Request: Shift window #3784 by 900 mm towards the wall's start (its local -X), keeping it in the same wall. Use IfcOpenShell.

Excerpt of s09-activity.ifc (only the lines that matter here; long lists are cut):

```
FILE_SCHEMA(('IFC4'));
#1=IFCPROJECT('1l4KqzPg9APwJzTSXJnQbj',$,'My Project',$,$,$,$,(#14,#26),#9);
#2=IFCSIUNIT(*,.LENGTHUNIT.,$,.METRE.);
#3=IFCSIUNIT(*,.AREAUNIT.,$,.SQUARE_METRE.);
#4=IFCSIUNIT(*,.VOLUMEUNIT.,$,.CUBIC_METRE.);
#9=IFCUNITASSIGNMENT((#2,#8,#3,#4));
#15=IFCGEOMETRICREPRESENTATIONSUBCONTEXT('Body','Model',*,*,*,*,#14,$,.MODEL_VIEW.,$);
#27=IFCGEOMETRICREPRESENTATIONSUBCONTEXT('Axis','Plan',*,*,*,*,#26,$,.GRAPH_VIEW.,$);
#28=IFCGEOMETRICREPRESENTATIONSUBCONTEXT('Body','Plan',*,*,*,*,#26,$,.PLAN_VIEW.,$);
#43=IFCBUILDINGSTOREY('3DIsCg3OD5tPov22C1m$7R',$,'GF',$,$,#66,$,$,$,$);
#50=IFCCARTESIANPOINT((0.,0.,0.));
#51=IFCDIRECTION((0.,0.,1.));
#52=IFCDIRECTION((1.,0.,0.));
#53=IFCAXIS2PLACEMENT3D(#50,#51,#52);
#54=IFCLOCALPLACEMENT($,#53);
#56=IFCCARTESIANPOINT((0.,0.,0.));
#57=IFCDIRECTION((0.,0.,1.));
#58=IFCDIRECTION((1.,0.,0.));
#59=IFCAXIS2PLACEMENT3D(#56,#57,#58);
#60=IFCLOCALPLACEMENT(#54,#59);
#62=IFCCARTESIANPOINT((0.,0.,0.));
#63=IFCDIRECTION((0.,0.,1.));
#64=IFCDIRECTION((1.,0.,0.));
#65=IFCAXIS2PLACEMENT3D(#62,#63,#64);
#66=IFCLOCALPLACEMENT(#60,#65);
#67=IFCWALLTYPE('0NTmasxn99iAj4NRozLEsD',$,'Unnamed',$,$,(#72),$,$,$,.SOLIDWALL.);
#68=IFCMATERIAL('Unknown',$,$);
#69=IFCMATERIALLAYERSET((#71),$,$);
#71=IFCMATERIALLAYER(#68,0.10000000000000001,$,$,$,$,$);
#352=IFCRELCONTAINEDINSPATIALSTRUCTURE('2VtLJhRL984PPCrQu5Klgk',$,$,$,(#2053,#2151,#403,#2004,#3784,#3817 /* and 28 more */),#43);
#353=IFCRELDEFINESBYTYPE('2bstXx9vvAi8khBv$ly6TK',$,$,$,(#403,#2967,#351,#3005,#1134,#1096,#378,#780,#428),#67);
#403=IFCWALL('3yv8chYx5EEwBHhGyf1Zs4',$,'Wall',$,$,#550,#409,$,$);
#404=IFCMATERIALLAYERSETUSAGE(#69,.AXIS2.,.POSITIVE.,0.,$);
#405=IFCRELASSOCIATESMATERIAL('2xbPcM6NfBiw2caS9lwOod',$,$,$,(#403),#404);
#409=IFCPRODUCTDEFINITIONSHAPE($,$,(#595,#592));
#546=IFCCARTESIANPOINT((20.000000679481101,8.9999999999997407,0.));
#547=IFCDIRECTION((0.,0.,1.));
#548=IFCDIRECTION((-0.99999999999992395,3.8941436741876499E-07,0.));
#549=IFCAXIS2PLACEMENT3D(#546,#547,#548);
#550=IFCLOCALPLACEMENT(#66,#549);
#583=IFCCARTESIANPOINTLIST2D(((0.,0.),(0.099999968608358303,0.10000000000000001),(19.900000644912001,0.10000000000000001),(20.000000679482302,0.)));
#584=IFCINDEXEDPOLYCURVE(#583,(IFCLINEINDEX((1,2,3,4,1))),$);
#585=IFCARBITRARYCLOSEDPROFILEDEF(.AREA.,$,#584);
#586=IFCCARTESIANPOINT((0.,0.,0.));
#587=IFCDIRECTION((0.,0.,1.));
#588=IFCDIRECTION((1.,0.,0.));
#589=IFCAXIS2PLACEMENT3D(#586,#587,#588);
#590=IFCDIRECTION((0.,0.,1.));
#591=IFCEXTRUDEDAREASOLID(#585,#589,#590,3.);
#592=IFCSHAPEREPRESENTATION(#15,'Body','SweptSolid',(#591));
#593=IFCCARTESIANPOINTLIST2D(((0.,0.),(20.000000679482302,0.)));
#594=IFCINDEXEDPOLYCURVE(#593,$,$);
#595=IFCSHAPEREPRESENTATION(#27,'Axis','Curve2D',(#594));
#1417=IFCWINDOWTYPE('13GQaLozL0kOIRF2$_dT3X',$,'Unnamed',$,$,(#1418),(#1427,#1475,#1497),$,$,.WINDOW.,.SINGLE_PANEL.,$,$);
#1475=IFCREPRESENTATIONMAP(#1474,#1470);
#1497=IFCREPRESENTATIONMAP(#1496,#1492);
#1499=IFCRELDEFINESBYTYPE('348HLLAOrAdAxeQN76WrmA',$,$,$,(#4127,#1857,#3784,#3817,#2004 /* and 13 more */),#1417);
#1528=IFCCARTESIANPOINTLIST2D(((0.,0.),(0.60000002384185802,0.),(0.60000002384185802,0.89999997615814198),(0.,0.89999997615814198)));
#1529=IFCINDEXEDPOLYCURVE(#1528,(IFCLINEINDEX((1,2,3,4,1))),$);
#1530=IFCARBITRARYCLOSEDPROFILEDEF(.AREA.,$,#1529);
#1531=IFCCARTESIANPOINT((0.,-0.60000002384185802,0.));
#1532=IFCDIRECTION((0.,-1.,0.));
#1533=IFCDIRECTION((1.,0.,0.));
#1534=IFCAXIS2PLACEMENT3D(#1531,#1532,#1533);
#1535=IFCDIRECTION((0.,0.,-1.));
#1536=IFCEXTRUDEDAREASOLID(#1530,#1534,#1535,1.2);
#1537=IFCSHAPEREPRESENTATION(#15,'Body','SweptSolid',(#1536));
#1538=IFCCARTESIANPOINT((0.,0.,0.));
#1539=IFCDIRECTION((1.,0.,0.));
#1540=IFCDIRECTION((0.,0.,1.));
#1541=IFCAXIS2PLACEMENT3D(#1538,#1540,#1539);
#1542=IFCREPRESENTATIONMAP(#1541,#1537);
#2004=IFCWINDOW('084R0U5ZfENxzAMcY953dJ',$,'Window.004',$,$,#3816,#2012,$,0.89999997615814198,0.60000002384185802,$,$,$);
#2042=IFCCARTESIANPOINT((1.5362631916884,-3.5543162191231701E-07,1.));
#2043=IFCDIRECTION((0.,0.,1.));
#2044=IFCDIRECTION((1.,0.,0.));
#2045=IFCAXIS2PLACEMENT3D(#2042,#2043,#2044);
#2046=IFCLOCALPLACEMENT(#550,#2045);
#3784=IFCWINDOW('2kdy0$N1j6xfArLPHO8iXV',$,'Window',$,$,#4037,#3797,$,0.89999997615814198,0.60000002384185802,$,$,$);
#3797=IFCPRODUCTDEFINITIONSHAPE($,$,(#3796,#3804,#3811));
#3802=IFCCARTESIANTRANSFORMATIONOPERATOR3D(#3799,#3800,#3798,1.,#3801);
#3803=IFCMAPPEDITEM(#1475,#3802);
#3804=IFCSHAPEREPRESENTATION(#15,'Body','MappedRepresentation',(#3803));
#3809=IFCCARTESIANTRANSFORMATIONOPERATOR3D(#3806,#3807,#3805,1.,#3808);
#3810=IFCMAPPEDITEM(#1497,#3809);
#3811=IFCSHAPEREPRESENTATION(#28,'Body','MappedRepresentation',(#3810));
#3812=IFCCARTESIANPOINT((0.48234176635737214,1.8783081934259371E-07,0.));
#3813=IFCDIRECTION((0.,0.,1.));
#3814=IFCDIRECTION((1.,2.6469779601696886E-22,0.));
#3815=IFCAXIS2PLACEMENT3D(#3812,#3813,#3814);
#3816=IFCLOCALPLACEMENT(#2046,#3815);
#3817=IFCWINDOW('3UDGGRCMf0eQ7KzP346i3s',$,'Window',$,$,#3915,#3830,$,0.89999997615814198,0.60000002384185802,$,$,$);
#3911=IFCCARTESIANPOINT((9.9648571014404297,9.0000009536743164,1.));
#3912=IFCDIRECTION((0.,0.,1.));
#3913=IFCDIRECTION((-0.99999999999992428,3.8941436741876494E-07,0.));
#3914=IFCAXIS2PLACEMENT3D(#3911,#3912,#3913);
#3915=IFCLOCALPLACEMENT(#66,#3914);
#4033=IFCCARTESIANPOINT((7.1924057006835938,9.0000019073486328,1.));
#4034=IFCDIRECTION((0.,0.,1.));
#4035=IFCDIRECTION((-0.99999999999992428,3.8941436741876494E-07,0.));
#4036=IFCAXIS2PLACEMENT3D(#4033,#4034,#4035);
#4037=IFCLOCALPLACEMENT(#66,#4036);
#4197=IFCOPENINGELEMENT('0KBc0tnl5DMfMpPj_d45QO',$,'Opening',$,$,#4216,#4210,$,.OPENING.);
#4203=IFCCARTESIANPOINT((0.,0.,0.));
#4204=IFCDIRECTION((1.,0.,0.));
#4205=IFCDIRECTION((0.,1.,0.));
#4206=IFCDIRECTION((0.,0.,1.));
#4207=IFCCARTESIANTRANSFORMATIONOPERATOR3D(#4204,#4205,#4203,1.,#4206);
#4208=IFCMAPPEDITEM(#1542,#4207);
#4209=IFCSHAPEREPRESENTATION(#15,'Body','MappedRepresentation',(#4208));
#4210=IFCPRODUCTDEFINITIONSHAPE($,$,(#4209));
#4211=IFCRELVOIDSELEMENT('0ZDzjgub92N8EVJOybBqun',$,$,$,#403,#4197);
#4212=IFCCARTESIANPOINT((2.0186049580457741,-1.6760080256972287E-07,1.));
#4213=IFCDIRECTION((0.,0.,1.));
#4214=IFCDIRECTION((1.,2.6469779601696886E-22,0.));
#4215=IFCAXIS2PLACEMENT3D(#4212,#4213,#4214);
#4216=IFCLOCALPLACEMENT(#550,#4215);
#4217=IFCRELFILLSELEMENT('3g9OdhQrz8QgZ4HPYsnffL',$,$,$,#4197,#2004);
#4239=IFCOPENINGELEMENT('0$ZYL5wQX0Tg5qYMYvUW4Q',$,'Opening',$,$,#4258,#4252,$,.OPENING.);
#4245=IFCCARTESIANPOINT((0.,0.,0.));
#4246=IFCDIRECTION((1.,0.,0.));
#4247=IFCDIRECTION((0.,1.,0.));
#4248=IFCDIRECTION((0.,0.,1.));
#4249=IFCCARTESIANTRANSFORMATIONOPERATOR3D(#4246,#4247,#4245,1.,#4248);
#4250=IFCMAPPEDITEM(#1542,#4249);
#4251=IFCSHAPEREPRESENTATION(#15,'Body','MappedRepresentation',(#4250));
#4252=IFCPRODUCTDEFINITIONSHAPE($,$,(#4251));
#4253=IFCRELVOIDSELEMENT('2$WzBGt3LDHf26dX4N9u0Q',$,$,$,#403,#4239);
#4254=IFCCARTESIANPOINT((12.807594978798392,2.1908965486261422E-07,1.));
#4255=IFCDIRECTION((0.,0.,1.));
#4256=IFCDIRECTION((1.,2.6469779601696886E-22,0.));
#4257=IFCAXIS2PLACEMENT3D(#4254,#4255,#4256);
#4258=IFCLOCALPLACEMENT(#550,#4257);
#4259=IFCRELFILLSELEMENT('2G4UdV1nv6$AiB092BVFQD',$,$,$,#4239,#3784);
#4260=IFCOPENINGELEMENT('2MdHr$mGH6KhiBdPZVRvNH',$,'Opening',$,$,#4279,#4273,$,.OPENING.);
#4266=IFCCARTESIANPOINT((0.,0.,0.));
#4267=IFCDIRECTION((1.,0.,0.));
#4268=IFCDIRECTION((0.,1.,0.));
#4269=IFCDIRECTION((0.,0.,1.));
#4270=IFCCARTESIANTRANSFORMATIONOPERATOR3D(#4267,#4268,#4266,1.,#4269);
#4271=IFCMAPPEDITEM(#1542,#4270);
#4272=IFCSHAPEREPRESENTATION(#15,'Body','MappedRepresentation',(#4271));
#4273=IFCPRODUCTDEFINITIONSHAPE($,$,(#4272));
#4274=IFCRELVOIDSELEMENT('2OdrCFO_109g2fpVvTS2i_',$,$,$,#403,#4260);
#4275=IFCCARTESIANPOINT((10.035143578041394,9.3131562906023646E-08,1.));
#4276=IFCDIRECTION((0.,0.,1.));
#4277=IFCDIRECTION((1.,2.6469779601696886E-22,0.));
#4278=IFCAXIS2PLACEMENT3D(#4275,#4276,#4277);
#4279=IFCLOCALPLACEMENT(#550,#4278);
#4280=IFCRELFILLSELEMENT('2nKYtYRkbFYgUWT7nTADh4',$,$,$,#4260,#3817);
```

```python
import ifcopenshell
import ifcopenshell.api.geometry
import ifcopenshell.util.placement
import ifcopenshell.util.unit

model = ifcopenshell.open("s09-activity.ifc")
unit_scale = ifcopenshell.util.unit.calculate_unit_scale(model)

window = model.by_guid("2kdy0$N1j6xfArLPHO8iXV")
opening = window.FillsVoids[0].RelatingOpeningElement
wall = opening.VoidsElements[0].RelatingBuildingElement

wall_matrix = ifcopenshell.util.placement.get_local_placement(wall.ObjectPlacement)
shift = wall_matrix[:3, 0] * -0.9 / unit_scale
before = ifcopenshell.util.placement.get_local_placement(window.ObjectPlacement)[:3, 3].copy()

# The window is not placed relative to its opening, so move both.
for product in (opening, window):
    matrix = ifcopenshell.util.placement.get_local_placement(product.ObjectPlacement)
    matrix[:3, 3] += shift
    ifcopenshell.api.geometry.edit_object_placement(model, product=product, matrix=matrix, is_si=False)

after = ifcopenshell.util.placement.get_local_placement(window.ObjectPlacement)[:3, 3]
print("window moved by", (after - before).round(3) + 0.0)

model.write("s09-activity_updated.ifc")
```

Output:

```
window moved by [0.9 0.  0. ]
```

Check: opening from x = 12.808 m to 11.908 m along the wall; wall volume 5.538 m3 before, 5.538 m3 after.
